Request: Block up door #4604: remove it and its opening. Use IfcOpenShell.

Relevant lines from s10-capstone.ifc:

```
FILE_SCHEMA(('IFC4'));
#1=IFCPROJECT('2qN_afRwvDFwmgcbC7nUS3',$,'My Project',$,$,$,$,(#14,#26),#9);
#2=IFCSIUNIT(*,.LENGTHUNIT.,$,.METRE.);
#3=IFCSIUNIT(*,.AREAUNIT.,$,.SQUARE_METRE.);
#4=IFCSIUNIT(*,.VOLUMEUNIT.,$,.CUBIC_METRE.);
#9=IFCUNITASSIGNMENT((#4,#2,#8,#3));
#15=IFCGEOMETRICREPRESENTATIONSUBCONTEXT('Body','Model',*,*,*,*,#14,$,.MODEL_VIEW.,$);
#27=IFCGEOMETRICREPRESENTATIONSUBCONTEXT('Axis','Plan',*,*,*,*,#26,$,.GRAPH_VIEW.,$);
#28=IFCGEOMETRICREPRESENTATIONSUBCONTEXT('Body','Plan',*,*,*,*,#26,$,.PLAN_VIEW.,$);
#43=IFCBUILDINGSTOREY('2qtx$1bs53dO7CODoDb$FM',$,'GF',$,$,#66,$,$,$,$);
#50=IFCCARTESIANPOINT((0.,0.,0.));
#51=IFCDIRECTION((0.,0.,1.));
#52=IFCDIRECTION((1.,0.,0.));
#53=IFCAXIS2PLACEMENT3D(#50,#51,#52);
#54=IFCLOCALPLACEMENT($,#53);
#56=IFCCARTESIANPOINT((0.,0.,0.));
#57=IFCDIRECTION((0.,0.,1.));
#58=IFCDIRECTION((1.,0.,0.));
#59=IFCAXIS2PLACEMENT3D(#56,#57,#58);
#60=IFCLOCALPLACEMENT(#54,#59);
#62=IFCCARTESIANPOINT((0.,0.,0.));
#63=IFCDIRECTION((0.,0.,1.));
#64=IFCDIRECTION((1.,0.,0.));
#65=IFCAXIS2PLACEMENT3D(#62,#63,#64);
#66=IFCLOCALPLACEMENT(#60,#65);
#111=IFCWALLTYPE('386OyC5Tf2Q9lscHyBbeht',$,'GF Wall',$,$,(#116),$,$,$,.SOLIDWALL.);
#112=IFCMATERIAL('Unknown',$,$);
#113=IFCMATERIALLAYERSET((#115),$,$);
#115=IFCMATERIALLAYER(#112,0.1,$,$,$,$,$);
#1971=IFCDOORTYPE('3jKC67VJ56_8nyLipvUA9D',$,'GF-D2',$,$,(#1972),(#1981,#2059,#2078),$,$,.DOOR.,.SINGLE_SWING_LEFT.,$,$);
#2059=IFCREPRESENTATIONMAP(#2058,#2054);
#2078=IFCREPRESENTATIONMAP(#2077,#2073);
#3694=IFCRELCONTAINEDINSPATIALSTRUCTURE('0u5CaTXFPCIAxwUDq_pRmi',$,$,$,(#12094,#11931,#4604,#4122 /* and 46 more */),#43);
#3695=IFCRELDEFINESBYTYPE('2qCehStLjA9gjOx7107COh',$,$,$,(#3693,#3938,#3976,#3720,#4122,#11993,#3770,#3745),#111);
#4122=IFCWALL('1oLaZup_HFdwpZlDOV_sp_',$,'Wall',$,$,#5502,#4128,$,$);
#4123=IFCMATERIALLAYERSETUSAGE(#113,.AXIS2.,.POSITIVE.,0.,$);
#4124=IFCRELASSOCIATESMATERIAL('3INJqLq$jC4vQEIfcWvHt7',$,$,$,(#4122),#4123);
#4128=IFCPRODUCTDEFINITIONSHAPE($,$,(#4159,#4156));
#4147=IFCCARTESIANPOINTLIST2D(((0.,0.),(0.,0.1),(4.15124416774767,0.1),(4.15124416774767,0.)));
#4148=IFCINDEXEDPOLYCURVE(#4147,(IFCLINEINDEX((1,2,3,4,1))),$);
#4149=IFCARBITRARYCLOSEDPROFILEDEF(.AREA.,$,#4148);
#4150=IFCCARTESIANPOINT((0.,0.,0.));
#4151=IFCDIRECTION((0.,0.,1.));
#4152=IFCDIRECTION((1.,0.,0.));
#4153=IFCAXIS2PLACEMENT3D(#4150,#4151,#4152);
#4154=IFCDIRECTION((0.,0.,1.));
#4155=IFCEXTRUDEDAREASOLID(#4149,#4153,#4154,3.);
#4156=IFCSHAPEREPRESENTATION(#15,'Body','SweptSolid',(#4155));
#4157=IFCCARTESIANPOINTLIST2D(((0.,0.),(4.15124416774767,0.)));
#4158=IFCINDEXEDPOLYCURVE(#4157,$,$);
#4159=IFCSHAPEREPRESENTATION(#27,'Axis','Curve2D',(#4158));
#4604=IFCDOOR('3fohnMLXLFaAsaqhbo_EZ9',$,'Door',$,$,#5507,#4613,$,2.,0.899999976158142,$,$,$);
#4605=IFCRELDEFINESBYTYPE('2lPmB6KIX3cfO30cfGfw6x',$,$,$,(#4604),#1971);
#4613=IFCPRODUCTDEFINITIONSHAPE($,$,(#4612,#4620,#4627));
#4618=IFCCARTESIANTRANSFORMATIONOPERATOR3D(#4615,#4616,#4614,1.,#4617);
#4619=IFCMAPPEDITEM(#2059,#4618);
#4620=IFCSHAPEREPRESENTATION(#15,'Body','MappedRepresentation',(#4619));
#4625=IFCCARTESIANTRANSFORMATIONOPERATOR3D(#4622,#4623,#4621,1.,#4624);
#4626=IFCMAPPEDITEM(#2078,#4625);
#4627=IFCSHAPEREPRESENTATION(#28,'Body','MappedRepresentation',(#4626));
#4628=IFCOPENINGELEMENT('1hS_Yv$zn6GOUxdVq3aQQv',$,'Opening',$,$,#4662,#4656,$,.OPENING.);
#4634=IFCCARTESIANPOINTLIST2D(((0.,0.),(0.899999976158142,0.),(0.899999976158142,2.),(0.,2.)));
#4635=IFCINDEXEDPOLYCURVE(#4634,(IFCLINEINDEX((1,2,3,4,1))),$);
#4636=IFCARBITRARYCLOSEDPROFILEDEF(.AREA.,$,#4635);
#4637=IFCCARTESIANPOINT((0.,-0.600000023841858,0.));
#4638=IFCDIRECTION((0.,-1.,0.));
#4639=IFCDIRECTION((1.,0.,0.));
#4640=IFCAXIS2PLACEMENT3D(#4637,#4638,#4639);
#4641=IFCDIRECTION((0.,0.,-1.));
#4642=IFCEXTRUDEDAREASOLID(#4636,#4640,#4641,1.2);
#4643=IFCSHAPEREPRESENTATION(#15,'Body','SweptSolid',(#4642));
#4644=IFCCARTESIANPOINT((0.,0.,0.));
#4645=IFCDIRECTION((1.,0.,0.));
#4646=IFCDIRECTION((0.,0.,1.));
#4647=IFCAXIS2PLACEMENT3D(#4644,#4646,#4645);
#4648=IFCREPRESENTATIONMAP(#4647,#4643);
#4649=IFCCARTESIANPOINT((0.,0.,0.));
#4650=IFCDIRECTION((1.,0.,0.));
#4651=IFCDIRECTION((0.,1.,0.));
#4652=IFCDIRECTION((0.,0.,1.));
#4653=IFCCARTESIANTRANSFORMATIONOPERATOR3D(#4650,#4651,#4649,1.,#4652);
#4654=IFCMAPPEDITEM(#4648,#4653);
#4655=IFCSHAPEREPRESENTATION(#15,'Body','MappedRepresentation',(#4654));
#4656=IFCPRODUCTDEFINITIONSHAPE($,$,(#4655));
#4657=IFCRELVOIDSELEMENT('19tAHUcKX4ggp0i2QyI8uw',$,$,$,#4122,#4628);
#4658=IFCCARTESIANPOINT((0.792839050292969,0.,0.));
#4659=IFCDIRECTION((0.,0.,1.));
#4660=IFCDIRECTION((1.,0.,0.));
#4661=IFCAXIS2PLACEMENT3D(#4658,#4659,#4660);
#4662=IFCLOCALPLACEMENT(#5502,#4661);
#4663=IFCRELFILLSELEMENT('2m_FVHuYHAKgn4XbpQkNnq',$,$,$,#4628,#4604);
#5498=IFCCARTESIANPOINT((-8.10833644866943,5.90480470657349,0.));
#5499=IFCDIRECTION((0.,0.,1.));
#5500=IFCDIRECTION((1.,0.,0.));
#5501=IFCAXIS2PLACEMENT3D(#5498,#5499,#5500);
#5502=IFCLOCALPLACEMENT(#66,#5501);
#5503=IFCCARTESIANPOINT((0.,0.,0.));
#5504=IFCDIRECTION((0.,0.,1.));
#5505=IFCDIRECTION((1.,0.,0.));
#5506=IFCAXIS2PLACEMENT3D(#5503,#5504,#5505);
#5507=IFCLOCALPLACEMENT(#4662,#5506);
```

```python
import ifcopenshell
import ifcopenshell.api.feature
import ifcopenshell.api.root
import ifcopenshell.geom
import ifcopenshell.util.shape

model = ifcopenshell.open("s10-capstone.ifc")
settings = ifcopenshell.geom.settings()


def volume(element):
    """Net volume in cubic metres, openings subtracted."""
    shape = ifcopenshell.geom.create_shape(settings, element)
    return ifcopenshell.util.shape.get_volume(shape.geometry)


door = model.by_guid("3fohnMLXLFaAsaqhbo_EZ9")
opening = door.FillsVoids[0].RelatingOpeningElement
wall = opening.VoidsElements[0].RelatingBuildingElement
before = volume(wall)

ifcopenshell.api.root.remove_product(model, product=door)
ifcopenshell.api.feature.remove_feature(model, feature=opening)

after = volume(wall)

print(f"wall volume {before:.3f} -> {after:.3f} m3")

model.write("s10-capstone-out.ifc")
```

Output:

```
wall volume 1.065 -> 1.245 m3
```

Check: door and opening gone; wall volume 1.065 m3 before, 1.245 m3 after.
